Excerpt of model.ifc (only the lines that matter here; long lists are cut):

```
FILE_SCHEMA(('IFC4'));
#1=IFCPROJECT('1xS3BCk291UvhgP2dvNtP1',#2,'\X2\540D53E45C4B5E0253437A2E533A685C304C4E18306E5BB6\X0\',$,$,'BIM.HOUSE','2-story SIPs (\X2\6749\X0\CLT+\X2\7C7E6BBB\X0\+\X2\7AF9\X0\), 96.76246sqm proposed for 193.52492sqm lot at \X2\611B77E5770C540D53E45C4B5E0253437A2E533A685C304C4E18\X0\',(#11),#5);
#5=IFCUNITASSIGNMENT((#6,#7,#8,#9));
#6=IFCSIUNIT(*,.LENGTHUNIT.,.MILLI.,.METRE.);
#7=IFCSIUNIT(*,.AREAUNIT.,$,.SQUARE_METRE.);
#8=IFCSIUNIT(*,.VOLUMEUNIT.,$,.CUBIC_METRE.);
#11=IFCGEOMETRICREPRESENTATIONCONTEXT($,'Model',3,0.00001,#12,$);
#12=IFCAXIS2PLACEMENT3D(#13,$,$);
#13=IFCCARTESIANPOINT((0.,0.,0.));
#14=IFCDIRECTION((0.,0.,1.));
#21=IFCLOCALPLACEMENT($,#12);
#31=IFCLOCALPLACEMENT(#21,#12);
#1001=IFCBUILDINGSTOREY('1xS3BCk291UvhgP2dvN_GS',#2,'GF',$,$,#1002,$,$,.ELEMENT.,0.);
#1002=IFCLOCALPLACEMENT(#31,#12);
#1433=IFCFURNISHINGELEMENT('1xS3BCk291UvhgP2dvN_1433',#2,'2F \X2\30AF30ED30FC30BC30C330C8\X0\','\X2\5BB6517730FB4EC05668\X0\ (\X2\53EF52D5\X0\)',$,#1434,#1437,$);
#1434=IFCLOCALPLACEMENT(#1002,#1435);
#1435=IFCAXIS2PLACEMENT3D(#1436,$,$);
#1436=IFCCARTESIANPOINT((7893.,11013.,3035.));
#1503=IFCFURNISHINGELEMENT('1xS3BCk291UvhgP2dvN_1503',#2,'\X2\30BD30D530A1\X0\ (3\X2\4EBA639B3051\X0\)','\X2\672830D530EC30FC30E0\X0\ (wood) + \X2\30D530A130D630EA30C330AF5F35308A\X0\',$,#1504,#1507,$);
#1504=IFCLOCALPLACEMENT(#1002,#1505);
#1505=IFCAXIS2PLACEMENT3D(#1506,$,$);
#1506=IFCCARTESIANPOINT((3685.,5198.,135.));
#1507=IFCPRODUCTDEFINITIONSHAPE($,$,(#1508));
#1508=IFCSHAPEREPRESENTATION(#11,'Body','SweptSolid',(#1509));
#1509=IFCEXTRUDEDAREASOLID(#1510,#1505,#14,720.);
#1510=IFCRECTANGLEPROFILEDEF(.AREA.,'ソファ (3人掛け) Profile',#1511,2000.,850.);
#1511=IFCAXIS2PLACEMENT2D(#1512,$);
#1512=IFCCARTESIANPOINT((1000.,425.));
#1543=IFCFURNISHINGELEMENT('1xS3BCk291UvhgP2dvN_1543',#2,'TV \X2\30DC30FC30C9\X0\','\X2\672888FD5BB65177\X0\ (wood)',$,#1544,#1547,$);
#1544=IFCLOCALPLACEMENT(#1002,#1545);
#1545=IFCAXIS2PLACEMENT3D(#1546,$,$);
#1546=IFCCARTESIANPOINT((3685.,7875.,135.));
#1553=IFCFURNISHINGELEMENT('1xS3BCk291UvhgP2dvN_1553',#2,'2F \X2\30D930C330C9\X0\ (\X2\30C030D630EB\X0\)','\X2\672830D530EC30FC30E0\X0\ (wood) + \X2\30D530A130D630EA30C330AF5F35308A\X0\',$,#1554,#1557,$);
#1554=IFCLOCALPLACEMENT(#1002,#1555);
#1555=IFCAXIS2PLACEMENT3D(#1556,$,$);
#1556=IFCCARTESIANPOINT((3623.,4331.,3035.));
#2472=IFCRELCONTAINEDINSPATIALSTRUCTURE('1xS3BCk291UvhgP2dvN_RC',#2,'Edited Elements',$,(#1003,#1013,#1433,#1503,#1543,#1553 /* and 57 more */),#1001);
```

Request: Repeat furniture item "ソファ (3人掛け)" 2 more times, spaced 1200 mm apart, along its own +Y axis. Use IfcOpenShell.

```python
import ifcopenshell
import ifcopenshell.api.geometry
import ifcopenshell.api.root
import ifcopenshell.util.element
import ifcopenshell.util.placement
import ifcopenshell.util.unit

model = ifcopenshell.open("model.ifc")
unit_scale = ifcopenshell.util.unit.calculate_unit_scale(model)


def reuse_history(source, copy):
    """copy_class also copies each property set's owner history, people and application; keep the originals."""
    for rel in copy.IsDefinedBy:
        if rel.is_a("IfcRelDefinesByProperties") and (history := rel.RelatingPropertyDefinition.OwnerHistory):
            rel.RelatingPropertyDefinition.OwnerHistory = source.OwnerHistory
            ifcopenshell.util.element.remove_deep2(model, history)


source = model.by_guid("1xS3BCk291UvhgP2dvN_1503")
base = ifcopenshell.util.placement.get_local_placement(source.ObjectPlacement)
step = base[:3, 1] * 1.2 / unit_scale

for i in range(1, 3):
    copy = ifcopenshell.api.root.copy_class(model, product=source)
    copy.Representation = ifcopenshell.util.element.copy_deep(
        model, source.Representation, exclude=["IfcGeometricRepresentationContext", "IfcRepresentationMap"]
    )
    reuse_history(source, copy)
    matrix = base.copy()
    matrix[:3, 3] += i * step
    print("added at", matrix[:3, 3].round(3) + 0.0)
    ifcopenshell.api.geometry.edit_object_placement(model, product=copy, matrix=matrix, is_si=False)

model.write("model_rev.ifc")
```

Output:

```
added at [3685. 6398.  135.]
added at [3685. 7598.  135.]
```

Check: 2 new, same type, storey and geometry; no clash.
